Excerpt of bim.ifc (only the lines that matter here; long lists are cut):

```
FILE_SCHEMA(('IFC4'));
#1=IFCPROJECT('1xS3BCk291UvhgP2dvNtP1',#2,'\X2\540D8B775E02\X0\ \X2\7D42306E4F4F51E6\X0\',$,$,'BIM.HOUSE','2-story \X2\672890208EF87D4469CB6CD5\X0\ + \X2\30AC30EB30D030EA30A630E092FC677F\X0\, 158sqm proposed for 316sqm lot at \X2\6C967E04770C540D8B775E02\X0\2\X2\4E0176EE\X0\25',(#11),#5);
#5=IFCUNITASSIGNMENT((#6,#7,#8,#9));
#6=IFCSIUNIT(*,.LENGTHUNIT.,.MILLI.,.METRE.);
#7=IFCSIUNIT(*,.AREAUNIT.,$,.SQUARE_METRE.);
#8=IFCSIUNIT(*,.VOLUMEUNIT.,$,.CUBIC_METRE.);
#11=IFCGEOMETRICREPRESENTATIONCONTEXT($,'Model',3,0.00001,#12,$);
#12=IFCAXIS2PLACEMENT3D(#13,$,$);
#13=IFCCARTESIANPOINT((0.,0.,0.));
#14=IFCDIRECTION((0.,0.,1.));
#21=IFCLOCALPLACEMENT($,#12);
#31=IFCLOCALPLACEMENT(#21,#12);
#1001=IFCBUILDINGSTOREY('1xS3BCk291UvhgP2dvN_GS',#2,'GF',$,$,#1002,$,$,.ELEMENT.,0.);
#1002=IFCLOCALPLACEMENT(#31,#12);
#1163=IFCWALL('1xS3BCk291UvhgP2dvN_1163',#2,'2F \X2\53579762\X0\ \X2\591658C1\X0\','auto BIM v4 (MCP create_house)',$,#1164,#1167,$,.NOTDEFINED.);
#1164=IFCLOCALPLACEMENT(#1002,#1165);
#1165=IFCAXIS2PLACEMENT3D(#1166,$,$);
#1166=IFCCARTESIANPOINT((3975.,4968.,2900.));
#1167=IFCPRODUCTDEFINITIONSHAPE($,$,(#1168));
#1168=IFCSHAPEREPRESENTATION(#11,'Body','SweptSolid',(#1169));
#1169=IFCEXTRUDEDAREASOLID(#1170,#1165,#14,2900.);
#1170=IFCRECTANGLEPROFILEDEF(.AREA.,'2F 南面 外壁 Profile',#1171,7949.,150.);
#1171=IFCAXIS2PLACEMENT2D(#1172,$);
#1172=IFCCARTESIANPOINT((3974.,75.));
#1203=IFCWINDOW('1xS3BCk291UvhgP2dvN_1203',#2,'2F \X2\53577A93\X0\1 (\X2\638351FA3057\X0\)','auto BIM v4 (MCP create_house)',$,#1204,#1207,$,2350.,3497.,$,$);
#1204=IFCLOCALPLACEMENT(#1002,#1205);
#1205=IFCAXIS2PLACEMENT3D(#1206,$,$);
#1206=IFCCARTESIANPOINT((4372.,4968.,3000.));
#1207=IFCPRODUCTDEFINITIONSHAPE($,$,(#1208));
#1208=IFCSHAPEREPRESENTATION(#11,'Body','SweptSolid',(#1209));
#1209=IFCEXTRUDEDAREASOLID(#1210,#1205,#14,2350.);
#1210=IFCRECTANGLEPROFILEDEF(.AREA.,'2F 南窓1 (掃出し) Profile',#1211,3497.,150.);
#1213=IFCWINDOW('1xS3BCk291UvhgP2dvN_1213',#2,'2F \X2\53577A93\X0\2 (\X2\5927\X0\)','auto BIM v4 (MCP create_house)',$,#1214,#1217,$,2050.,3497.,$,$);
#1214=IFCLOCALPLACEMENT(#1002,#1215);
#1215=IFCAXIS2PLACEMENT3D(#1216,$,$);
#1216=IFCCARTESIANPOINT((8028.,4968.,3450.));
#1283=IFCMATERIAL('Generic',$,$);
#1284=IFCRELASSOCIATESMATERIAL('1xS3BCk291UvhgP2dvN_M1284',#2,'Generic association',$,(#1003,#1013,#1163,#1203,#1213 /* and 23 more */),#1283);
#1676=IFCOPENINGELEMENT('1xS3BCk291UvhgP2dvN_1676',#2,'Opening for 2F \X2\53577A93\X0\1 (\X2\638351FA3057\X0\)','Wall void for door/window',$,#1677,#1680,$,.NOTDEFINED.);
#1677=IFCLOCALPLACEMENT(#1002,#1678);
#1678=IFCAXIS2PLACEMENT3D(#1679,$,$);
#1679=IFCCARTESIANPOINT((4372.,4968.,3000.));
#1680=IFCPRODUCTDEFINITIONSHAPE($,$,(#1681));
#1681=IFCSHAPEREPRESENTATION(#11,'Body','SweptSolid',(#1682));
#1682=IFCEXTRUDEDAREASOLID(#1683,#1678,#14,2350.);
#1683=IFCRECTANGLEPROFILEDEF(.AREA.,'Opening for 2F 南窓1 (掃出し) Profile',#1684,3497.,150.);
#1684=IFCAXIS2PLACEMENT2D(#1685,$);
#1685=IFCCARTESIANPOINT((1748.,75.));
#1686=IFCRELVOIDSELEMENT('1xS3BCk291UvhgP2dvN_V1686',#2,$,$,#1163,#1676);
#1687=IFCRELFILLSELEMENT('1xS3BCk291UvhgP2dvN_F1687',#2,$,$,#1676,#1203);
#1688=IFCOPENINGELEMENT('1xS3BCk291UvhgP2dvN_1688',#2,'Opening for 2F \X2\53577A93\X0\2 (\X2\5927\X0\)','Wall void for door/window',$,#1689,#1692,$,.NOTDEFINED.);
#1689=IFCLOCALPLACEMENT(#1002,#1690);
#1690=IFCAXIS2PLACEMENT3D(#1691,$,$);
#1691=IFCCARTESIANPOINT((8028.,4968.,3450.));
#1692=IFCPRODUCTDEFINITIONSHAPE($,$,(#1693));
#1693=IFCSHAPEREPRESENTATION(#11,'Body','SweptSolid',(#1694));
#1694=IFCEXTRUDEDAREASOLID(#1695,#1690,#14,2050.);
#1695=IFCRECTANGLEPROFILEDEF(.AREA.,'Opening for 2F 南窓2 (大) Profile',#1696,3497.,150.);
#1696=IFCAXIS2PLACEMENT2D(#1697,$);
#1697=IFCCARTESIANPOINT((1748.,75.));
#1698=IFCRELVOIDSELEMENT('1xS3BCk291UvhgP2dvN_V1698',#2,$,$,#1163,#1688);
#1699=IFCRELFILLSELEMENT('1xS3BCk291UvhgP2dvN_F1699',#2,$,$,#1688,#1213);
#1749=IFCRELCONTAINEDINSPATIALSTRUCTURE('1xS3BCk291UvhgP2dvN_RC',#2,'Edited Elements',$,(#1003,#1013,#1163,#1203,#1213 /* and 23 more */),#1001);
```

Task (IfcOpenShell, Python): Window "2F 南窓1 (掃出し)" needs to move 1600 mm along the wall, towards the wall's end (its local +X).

```python
import ifcopenshell
import ifcopenshell.api.geometry
import ifcopenshell.util.placement

model = ifcopenshell.open("bim.ifc")

window = model.by_guid("1xS3BCk291UvhgP2dvN_1203")
opening = window.FillsVoids[0].RelatingOpeningElement
wall = opening.VoidsElements[0].RelatingBuildingElement

wall_matrix = ifcopenshell.util.placement.get_local_placement(wall.ObjectPlacement)
shift = wall_matrix[:3, 0] * 1600.0
before = ifcopenshell.util.placement.get_local_placement(window.ObjectPlacement)[:3, 3].copy()

# The window is not placed relative to its opening, so move both.
for product in (opening, window):
    matrix = ifcopenshell.util.placement.get_local_placement(product.ObjectPlacement)
    matrix[:3, 3] += shift
    ifcopenshell.api.geometry.edit_object_placement(model, product=product, matrix=matrix, is_si=False)

after = ifcopenshell.util.placement.get_local_placement(window.ObjectPlacement)[:3, 3]
print("window moved by", (after - before).round(3) + 0.0)

model.write("bim_updated.ifc")
```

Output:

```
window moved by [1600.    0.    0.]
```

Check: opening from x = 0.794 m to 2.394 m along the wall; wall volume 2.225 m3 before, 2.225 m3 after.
